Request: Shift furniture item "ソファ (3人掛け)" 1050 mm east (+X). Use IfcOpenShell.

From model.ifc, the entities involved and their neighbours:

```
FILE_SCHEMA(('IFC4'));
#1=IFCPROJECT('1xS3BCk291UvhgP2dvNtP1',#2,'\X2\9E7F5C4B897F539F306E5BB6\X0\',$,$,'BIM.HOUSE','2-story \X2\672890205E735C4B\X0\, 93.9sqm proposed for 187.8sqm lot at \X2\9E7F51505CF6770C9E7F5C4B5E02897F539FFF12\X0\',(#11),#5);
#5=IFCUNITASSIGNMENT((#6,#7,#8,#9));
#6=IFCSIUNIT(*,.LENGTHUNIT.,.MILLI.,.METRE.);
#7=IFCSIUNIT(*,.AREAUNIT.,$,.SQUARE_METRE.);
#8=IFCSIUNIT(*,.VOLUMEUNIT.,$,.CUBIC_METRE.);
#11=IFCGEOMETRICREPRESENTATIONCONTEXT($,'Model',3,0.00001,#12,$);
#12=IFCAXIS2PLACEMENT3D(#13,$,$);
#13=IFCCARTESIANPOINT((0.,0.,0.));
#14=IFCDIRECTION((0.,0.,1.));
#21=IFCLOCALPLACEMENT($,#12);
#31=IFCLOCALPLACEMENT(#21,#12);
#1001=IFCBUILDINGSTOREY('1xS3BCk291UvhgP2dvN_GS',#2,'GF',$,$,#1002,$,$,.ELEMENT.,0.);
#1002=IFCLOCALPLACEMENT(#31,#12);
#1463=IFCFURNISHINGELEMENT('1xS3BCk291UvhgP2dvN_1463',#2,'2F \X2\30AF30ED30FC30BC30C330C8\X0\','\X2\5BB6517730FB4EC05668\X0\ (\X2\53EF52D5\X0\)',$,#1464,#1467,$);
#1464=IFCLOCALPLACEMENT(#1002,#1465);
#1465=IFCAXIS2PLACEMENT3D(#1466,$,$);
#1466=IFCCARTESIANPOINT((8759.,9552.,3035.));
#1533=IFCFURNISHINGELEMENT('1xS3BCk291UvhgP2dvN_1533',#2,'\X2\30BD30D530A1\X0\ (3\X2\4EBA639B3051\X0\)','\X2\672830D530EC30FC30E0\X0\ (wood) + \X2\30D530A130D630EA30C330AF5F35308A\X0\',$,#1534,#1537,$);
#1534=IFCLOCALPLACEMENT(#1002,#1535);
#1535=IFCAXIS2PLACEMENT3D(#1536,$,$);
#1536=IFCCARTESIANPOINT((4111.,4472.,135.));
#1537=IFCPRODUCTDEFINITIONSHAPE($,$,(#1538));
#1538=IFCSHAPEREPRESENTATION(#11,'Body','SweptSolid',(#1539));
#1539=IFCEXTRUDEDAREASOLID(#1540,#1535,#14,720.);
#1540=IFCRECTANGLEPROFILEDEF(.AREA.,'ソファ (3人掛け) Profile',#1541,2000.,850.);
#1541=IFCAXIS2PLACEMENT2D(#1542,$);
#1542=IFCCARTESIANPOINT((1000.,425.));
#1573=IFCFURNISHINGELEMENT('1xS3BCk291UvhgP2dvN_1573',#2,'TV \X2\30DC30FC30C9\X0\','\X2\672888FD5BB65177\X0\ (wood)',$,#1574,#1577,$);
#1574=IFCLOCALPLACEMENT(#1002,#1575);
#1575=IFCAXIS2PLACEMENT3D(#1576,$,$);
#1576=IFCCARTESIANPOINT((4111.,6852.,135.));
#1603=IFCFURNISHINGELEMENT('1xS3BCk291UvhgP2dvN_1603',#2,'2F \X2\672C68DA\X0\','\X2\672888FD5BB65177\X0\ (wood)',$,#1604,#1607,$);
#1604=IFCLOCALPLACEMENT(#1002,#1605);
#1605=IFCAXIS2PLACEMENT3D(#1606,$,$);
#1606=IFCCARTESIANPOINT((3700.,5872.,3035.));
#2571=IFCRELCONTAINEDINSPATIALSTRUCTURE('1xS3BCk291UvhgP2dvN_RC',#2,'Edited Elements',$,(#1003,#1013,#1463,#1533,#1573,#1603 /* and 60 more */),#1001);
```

```python
import ifcopenshell
import ifcopenshell.api.geometry
import ifcopenshell.util.placement
import ifcopenshell.util.unit

model = ifcopenshell.open("model.ifc")
unit_scale = ifcopenshell.util.unit.calculate_unit_scale(model)

item = model.by_id(1533)
matrix = ifcopenshell.util.placement.get_local_placement(item.ObjectPlacement)
matrix[0, 3] += 1.05 / unit_scale
ifcopenshell.api.geometry.edit_object_placement(model, product=item, matrix=matrix, is_si=False)

print(ifcopenshell.util.placement.get_local_placement(item.ObjectPlacement).round(3) + 0.0)

model.write("model_v2.ifc")
```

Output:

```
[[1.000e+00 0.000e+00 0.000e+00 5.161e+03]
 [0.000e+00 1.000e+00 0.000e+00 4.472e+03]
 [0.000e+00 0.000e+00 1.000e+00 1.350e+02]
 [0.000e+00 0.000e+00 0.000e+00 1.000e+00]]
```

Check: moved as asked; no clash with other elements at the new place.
